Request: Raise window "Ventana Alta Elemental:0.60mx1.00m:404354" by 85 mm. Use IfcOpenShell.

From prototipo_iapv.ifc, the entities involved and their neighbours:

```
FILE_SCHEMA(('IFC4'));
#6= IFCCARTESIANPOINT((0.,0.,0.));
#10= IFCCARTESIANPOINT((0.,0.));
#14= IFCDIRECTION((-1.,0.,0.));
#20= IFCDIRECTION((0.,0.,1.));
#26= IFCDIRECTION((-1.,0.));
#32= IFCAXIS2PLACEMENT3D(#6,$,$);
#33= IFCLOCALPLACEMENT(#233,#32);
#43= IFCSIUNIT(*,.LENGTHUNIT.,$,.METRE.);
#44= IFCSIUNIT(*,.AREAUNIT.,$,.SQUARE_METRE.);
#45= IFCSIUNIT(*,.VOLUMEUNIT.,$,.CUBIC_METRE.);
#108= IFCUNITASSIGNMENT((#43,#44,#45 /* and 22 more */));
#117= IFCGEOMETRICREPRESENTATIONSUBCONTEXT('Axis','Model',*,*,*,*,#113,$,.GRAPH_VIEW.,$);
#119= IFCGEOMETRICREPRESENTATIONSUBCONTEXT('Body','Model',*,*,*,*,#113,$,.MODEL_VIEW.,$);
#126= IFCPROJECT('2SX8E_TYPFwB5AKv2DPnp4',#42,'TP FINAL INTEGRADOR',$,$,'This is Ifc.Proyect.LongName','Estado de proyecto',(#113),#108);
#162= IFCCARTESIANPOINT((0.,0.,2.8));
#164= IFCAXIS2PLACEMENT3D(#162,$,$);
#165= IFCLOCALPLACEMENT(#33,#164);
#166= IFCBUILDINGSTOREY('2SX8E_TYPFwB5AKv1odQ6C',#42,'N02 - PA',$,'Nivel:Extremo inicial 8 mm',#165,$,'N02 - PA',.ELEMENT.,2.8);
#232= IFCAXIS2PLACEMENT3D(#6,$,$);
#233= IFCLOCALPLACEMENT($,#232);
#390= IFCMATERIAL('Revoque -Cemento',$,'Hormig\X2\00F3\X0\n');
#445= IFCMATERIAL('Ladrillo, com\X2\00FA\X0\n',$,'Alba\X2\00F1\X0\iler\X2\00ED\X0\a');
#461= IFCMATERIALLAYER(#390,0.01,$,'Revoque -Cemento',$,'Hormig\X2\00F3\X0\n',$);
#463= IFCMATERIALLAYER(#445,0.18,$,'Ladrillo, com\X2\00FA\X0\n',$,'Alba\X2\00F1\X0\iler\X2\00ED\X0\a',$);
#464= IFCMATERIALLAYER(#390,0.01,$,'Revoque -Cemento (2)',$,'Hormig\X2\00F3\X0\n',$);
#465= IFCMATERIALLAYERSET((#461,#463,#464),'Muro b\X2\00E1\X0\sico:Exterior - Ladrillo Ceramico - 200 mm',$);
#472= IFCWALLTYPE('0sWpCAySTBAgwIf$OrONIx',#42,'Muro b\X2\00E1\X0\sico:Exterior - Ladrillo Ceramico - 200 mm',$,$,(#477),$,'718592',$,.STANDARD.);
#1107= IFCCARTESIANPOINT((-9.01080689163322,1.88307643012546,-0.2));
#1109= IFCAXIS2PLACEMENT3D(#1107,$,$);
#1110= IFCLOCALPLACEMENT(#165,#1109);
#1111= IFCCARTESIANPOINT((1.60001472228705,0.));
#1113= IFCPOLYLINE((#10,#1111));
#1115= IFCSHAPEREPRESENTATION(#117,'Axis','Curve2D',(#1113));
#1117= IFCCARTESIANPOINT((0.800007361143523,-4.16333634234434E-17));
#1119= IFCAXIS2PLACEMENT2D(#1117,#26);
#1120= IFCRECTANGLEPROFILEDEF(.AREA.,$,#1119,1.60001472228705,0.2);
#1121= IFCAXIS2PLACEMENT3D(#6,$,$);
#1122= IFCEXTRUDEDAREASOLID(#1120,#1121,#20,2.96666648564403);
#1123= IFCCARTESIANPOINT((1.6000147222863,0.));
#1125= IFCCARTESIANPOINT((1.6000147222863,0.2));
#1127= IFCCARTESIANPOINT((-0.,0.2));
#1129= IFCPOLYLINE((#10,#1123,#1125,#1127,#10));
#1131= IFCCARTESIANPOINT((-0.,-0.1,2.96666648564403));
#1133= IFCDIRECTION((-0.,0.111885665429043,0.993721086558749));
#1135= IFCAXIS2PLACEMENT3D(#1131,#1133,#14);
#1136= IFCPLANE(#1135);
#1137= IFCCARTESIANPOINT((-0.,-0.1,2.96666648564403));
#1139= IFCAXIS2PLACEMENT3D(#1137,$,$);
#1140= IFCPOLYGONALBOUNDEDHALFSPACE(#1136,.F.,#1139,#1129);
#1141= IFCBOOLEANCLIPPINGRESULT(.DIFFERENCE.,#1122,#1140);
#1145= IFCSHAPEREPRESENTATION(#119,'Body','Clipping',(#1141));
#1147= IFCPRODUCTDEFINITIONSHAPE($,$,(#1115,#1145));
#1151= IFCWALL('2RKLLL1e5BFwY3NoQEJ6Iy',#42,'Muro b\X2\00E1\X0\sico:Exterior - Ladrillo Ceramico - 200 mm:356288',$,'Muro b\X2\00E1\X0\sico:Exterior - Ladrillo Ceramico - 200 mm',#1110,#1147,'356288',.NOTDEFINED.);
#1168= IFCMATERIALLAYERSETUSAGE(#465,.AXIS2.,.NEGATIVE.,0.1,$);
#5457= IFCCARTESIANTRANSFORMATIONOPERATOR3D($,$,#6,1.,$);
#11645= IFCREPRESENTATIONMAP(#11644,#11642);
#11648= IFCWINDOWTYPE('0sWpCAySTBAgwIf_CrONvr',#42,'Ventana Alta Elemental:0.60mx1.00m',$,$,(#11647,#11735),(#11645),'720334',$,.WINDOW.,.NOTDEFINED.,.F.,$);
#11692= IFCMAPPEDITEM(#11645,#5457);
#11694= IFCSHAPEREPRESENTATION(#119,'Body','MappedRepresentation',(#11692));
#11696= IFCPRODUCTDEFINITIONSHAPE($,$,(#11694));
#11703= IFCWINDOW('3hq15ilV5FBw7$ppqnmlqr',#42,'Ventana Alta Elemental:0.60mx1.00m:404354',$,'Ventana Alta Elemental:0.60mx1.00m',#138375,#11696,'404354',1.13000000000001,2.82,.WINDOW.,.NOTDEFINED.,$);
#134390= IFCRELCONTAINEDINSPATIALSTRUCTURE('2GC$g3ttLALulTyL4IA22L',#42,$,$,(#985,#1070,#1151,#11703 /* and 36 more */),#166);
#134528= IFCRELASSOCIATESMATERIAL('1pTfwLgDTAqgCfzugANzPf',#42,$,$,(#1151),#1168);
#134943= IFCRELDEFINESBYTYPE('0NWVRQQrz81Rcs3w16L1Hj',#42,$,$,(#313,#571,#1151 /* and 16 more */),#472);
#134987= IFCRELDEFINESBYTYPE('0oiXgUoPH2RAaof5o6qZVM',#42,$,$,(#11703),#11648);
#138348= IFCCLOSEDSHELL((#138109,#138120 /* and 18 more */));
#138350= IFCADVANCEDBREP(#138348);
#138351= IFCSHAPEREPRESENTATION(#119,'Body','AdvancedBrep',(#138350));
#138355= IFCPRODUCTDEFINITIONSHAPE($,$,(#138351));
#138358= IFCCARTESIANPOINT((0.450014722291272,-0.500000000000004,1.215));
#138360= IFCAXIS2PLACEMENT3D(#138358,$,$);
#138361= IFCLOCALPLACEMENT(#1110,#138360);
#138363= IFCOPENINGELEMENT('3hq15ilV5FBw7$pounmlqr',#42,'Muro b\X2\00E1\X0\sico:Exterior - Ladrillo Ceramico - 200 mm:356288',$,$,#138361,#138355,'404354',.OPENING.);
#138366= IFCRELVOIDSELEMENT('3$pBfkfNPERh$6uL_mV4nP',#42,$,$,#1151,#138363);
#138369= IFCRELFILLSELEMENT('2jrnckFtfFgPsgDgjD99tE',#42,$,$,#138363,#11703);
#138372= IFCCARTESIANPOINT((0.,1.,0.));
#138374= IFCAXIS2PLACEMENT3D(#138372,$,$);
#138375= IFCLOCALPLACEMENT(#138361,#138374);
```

```python
import numpy as np
import ifcopenshell
import ifcopenshell.api.geometry
import ifcopenshell.util.placement
import ifcopenshell.util.unit

model = ifcopenshell.open("prototipo_iapv.ifc")
unit_scale = ifcopenshell.util.unit.calculate_unit_scale(model)

window = model.by_id(11703)
opening = window.FillsVoids[0].RelatingOpeningElement
dz = 0.085 / unit_scale

shift = np.array([0.0, 0.0, dz])
# The window is placed relative to its opening, so it follows when the opening moves.
matrix = ifcopenshell.util.placement.get_local_placement(opening.ObjectPlacement)
matrix[:3, 3] += shift
ifcopenshell.api.geometry.edit_object_placement(
    model, product=opening, matrix=matrix, is_si=False, should_transform_children=True
)

print(f"moved by {dz * unit_scale:+.3f} m")

model.write("prototipo_iapv_edited.ifc")
```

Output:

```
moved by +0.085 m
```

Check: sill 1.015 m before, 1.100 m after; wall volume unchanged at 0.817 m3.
